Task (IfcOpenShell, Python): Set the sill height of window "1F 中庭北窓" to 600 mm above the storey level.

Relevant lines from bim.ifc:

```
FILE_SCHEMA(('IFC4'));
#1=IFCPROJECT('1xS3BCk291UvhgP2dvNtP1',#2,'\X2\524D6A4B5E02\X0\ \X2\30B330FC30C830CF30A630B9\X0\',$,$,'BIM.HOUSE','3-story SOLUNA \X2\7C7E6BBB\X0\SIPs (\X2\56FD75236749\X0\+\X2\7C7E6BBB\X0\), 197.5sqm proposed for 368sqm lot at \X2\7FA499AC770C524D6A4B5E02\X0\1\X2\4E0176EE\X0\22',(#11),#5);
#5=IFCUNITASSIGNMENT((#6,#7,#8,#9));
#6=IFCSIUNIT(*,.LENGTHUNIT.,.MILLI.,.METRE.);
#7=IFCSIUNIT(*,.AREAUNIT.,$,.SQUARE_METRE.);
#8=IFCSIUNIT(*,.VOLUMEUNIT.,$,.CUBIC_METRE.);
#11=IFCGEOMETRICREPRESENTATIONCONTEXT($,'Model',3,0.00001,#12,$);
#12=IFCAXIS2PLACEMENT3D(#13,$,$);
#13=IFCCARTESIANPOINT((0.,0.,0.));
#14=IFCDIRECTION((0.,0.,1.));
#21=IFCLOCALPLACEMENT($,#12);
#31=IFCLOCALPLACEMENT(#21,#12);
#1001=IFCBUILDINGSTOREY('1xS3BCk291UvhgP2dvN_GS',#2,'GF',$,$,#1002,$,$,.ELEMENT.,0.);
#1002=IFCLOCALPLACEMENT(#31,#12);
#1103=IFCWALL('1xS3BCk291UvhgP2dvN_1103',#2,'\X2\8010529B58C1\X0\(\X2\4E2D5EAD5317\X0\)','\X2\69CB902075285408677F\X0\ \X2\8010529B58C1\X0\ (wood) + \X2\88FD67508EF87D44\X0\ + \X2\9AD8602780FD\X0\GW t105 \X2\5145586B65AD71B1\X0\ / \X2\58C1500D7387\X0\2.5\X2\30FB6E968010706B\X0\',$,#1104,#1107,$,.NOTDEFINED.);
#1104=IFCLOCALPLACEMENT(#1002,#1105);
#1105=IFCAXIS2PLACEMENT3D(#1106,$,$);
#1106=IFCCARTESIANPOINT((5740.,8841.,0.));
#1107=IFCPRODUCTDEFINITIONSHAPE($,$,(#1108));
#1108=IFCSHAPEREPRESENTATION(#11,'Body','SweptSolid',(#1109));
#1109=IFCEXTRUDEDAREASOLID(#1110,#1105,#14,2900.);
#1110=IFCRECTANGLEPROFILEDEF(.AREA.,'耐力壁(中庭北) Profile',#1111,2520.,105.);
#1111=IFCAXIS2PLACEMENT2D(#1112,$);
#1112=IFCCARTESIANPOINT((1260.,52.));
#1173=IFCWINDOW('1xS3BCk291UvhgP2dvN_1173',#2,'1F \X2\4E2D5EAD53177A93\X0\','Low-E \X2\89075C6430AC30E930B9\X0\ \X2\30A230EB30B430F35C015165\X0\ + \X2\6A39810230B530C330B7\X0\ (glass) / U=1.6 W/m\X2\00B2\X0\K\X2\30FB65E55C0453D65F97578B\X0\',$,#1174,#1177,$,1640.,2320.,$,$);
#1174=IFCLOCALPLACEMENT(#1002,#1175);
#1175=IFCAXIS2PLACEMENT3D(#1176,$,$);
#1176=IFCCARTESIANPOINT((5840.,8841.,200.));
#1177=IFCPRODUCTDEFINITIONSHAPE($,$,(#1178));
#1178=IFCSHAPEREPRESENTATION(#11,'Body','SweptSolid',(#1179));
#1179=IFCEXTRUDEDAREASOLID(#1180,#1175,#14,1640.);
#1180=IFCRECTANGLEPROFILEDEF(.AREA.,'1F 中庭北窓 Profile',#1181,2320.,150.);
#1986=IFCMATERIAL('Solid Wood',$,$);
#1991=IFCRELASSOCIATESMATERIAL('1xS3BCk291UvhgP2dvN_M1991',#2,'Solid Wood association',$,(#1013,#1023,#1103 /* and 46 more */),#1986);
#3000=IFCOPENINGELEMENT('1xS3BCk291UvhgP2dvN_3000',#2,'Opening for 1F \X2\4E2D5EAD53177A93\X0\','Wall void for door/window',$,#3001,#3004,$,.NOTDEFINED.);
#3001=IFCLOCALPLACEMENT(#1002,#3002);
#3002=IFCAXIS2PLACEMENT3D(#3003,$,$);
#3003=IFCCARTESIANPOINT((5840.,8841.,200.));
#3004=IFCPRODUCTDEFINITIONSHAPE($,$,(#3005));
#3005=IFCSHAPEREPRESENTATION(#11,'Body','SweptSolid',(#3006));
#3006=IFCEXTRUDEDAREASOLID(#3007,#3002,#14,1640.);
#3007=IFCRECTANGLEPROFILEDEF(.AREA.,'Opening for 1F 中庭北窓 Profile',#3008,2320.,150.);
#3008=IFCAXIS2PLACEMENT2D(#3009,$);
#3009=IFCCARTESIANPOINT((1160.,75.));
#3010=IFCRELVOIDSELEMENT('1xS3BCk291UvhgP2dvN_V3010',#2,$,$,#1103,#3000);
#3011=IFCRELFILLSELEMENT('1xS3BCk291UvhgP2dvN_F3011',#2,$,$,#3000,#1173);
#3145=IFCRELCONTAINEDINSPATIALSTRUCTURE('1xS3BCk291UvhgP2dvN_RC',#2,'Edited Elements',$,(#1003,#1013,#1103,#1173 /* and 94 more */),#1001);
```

```python
import numpy as np
import ifcopenshell
import ifcopenshell.api.geometry
import ifcopenshell.geom
import ifcopenshell.util.element
import ifcopenshell.util.placement
import ifcopenshell.util.shape
import ifcopenshell.util.unit

model = ifcopenshell.open("bim.ifc")
unit_scale = ifcopenshell.util.unit.calculate_unit_scale(model)

window = model.by_guid("1xS3BCk291UvhgP2dvN_1173")
opening = window.FillsVoids[0].RelatingOpeningElement
storey = ifcopenshell.util.element.get_container(window, ifc_class="IfcBuildingStorey")
level = ifcopenshell.util.placement.get_local_placement(storey.ObjectPlacement)[2, 3]

# The opening's origin need not be at the sill, so measure its lowest point.
shape = ifcopenshell.geom.create_shape(ifcopenshell.geom.settings(), opening)
bottom = ifcopenshell.util.shape.get_shape_bottom_elevation(shape, shape.geometry) / unit_scale
dz = level + 0.6 / unit_scale - bottom

shift = np.array([0.0, 0.0, dz])
# The window is not placed relative to its opening, so move both.
for product in (opening, window):
    matrix = ifcopenshell.util.placement.get_local_placement(product.ObjectPlacement)
    matrix[:3, 3] += shift
    ifcopenshell.api.geometry.edit_object_placement(model, product=product, matrix=matrix, is_si=False)

print(f"moved by {dz * unit_scale:+.3f} m")

model.write("bim-out.ifc")
```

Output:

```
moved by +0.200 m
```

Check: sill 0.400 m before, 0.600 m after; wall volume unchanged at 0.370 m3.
